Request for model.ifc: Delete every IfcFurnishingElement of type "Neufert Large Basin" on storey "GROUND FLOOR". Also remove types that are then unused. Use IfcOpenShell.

First a look at what the model holds.

```python
import ifcopenshell
import ifcopenshell.util.element

model = ifcopenshell.open("model.ifc")
print(model.schema)
storey = next(s for s in model.by_type("IfcBuildingStorey") if s.Name == "GROUND FLOOR")
furniture = [e for e in ifcopenshell.util.element.get_decomposition(storey) if e.is_a("IfcFurnishingElement")]
seen = {}
for e in furniture:
    element_type = ifcopenshell.util.element.get_type(e)
    name = element_type.Name if element_type not in (None, e) else None
    seen[name] = seen.get(name, 0) + 1
for name, count in sorted(seen.items(), key=str):
    print(count, "x", name)
```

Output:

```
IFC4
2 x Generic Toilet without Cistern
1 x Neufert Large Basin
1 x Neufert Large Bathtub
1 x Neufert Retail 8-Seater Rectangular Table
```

```python
import ifcopenshell
import ifcopenshell.api.root
import ifcopenshell.util.element

model = ifcopenshell.open("model.ifc")

storey = next(s for s in model.by_type("IfcBuildingStorey") if s.Name == "GROUND FLOOR")
furniture = [e for e in ifcopenshell.util.element.get_decomposition(storey) if e.is_a("IfcFurnishingElement")]
targets = [e for e in furniture if (t := ifcopenshell.util.element.get_type(e)) not in (None, e) and t.Name == "Neufert Large Basin"]
types = {ifcopenshell.util.element.get_type(e) for e in targets} - {None, *targets}

for e in targets:
    ifcopenshell.api.root.remove_product(model, product=e)
print(len(targets), "removed")

unused = [t for t in types if not ifcopenshell.util.element.get_types(t)]
for t in unused:
    ifcopenshell.api.root.remove_product(model, product=t)
print(len(unused), "unused types removed")

model.write("model_v2.ifc")
```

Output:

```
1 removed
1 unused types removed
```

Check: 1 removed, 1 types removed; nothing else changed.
